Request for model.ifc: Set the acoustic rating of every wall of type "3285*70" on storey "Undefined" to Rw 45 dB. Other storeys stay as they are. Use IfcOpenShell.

First a look at what the model holds.

```python
import ifcopenshell
import ifcopenshell.util.element

model = ifcopenshell.open("model.ifc")
print(model.schema)
storey = next(s for s in model.by_type("IfcBuildingStorey") if s.Name == "Undefined")
walls = [e for e in ifcopenshell.util.element.get_decomposition(storey) if e.is_a("IfcWall")]
seen = {}
for e in walls:
    element_type = ifcopenshell.util.element.get_type(e)
    key = (element_type.Name if element_type != e and element_type else None, ifcopenshell.util.element.get_pset(e, "Pset_WallCommon", "AcousticRating"))
    seen[key] = seen.get(key, 0) + 1
for (name, value), count in sorted(seen.items(), key=str):
    print(count, "x", name, "|", value)
```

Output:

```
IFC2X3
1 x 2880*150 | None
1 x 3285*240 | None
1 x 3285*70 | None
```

```python
import ifcopenshell
import ifcopenshell.api.pset
import ifcopenshell.util.element

model = ifcopenshell.open("model.ifc")

storey = next(s for s in model.by_type("IfcBuildingStorey") if s.Name == "Undefined")
walls = [e for e in ifcopenshell.util.element.get_decomposition(storey) if e.is_a("IfcWall")]

count = 0
for e in walls:
    element_type = ifcopenshell.util.element.get_type(e)
    if element_type in (None, e) or element_type.Name != "3285*70":
        continue
    # add_pset returns the element's existing set when there is one.
    pset = ifcopenshell.api.pset.add_pset(model, product=e, name="Pset_WallCommon")
    ifcopenshell.api.pset.edit_pset(model, pset=pset, properties={"AcousticRating": "Rw 45 dB"})
    count += 1

print(count, "walls updated")

model.write("model_rev.ifc")
```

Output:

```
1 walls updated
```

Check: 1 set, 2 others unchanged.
